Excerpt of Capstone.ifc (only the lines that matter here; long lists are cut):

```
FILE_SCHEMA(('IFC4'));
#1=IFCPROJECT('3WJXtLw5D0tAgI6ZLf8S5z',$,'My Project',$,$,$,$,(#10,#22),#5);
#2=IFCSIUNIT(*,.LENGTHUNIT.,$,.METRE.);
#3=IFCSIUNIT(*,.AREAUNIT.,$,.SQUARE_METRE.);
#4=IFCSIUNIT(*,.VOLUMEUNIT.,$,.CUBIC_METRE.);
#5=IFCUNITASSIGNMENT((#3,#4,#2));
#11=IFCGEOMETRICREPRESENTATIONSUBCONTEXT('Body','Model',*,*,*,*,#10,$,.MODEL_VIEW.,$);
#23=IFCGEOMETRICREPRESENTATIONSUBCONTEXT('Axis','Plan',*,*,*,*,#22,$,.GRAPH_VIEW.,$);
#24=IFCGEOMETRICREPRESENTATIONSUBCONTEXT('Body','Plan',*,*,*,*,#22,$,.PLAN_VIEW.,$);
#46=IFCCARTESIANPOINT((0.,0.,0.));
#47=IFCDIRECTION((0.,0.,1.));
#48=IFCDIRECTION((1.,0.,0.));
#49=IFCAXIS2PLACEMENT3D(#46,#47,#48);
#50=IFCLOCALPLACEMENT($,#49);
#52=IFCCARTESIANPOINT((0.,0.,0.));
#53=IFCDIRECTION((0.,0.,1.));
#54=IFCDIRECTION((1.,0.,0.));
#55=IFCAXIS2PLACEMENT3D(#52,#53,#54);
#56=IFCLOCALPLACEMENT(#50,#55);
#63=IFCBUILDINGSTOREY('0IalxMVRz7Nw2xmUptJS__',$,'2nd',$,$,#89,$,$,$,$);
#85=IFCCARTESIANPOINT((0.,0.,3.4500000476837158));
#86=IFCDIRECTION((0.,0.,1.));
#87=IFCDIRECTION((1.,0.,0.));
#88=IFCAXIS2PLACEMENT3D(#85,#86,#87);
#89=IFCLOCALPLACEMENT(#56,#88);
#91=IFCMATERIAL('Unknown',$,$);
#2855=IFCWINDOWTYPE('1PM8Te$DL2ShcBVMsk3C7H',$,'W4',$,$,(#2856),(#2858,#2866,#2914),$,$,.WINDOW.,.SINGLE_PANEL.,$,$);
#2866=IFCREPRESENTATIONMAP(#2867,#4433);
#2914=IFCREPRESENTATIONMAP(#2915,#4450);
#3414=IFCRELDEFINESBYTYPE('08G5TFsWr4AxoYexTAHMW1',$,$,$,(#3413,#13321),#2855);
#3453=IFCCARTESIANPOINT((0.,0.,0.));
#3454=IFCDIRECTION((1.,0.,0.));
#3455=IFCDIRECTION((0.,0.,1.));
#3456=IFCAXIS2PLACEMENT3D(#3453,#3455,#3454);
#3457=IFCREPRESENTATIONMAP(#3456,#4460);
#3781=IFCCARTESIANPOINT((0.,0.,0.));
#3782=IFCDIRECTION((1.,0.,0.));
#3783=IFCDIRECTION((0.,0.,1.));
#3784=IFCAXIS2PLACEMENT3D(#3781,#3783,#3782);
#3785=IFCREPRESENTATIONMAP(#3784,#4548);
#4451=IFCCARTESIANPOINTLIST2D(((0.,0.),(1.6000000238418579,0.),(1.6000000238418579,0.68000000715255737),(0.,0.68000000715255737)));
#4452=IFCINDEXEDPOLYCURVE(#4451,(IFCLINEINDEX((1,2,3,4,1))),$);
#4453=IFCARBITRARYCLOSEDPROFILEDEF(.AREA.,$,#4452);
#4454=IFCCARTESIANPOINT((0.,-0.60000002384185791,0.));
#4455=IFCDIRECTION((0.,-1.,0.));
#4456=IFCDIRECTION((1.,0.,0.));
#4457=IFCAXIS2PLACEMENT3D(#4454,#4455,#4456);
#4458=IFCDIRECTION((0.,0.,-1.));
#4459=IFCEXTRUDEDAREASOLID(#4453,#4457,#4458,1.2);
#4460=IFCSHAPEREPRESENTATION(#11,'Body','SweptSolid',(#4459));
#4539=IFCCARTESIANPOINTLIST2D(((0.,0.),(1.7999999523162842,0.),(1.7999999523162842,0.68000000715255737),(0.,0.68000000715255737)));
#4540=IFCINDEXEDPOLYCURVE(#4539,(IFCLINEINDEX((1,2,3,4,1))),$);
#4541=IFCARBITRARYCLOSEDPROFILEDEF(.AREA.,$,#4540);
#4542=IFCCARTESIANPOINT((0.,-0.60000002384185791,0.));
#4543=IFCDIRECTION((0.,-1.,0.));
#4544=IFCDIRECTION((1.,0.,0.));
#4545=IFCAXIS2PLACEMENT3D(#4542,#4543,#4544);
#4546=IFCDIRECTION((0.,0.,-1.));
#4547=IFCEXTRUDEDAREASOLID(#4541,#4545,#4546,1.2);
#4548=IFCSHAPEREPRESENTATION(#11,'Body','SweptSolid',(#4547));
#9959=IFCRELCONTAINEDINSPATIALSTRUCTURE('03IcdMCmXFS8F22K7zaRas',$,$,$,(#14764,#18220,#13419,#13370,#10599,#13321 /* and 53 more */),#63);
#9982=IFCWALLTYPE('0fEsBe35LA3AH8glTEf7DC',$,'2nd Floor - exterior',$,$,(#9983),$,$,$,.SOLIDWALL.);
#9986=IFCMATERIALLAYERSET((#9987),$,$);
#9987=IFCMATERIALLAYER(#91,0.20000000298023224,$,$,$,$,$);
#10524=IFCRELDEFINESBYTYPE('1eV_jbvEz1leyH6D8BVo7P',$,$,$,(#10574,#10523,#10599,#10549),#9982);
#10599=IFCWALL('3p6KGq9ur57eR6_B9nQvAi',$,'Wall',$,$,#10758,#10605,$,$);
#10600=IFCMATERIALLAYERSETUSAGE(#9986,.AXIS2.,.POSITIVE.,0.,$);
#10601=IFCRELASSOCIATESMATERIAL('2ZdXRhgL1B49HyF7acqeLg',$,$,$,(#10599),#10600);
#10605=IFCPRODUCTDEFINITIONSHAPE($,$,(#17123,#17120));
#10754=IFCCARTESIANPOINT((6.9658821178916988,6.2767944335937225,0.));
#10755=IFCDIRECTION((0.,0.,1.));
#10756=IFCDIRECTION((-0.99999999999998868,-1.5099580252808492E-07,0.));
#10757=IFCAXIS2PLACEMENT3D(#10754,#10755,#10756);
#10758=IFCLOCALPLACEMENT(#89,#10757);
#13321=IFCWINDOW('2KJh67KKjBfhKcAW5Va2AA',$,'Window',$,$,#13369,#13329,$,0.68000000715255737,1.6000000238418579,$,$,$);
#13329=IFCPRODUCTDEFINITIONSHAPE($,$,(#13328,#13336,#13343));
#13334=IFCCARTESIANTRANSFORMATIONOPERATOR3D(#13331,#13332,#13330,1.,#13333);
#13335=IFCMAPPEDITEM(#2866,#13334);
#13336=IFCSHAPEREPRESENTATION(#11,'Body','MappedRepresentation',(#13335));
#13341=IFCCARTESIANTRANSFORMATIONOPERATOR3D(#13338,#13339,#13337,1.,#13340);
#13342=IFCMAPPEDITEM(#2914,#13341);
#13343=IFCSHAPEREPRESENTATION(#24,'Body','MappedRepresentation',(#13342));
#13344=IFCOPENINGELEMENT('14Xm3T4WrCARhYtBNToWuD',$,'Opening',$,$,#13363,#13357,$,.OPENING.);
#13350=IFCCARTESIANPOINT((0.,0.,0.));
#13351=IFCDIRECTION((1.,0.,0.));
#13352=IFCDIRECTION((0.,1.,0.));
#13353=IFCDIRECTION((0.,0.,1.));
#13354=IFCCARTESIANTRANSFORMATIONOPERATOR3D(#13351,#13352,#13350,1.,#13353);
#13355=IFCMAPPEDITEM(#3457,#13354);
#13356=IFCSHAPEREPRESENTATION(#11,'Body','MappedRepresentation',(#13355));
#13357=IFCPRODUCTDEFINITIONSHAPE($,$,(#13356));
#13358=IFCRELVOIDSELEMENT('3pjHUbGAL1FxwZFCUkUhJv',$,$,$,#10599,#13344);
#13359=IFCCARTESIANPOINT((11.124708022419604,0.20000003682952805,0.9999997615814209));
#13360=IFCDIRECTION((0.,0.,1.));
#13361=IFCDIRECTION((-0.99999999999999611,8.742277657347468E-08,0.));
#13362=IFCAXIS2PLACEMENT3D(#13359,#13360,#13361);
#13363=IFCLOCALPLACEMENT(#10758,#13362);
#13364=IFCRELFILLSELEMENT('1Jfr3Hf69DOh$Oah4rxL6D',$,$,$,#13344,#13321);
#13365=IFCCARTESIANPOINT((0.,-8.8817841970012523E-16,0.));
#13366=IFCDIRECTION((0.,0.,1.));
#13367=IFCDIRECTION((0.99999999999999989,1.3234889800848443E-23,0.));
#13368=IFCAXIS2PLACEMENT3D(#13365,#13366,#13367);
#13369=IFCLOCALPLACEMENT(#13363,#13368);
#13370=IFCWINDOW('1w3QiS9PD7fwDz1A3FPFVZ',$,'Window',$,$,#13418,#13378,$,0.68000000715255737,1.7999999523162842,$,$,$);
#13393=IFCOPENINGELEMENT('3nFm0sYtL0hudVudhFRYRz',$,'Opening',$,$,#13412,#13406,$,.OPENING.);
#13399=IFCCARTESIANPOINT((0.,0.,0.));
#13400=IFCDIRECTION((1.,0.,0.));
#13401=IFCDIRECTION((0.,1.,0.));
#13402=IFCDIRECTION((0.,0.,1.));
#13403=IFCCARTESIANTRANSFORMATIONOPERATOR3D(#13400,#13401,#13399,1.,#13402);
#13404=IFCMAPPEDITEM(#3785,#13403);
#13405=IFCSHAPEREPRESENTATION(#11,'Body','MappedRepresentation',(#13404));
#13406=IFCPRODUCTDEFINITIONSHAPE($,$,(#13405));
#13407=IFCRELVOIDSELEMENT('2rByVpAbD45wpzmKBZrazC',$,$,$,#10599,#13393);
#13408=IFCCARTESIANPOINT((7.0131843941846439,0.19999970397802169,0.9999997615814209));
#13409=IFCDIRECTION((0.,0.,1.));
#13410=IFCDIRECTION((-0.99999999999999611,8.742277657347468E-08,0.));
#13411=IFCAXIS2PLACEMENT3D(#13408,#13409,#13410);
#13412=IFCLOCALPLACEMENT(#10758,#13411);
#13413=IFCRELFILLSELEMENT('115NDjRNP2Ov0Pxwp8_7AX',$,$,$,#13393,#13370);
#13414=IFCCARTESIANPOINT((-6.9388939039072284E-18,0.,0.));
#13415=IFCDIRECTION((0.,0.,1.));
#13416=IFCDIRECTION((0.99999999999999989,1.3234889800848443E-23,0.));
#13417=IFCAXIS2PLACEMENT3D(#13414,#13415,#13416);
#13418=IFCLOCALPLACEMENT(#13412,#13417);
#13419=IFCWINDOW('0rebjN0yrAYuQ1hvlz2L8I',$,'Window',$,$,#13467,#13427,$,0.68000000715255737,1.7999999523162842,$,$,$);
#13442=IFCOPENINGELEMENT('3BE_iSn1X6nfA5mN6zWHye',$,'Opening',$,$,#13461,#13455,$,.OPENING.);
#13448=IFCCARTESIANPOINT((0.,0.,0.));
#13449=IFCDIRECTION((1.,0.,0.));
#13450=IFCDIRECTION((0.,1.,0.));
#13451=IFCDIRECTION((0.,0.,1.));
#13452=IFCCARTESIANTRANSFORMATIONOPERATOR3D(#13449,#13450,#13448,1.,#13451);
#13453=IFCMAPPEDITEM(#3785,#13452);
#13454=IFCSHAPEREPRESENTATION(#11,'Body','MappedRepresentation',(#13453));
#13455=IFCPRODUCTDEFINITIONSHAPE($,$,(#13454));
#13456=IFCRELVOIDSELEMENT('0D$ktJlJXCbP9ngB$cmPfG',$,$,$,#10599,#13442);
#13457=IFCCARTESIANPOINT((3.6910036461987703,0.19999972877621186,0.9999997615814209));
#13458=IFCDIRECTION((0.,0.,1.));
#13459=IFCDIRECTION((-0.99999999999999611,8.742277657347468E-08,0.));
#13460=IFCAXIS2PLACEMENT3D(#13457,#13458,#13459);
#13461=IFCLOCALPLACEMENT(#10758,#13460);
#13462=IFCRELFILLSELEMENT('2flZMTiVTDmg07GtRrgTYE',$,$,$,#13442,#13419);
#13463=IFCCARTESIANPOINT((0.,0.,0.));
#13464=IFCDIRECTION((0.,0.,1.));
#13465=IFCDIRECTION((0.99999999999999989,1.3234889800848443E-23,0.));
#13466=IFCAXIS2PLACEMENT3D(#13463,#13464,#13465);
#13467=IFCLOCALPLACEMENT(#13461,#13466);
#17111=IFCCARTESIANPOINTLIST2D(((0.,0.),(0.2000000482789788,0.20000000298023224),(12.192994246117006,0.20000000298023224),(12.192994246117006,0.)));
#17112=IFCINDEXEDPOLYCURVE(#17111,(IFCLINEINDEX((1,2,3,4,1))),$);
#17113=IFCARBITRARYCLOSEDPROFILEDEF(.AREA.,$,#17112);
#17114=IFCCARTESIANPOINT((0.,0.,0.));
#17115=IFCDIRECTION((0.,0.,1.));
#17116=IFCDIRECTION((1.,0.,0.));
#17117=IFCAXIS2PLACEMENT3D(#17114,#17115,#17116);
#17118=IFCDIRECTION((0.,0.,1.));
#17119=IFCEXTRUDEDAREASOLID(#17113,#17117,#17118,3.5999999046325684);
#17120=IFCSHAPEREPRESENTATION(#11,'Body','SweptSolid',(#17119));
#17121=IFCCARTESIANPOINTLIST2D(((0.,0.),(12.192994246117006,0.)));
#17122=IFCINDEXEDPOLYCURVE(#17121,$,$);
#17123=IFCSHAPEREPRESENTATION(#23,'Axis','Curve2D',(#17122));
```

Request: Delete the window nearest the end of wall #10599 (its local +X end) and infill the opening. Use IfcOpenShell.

```python
import ifcopenshell
import ifcopenshell.api.feature
import ifcopenshell.api.root
import ifcopenshell.geom
import ifcopenshell.util.shape

model = ifcopenshell.open("Capstone.ifc")
settings = ifcopenshell.geom.settings()


def volume(element):
    """Net volume in cubic metres, openings subtracted."""
    shape = ifcopenshell.geom.create_shape(settings, element)
    return ifcopenshell.util.shape.get_volume(shape.geometry)


window = model.by_guid("2KJh67KKjBfhKcAW5Va2AA")
opening = window.FillsVoids[0].RelatingOpeningElement
wall = opening.VoidsElements[0].RelatingBuildingElement
before = volume(wall)

ifcopenshell.api.root.remove_product(model, product=window)
ifcopenshell.api.feature.remove_feature(model, feature=opening)

after = volume(wall)

print(f"wall volume {before:.3f} -> {after:.3f} m3")

model.write("Capstone_v2.ifc")
```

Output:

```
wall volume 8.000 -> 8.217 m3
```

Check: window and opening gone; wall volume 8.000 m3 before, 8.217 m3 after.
